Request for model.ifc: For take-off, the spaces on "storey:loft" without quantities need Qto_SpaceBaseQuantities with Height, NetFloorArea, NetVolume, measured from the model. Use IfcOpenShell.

First a look at what the model holds.

```python
import ifcopenshell
import ifcopenshell.util.element
import ifcopenshell.util.unit

model = ifcopenshell.open("model.ifc")
print(model.schema)
for unit_type in ("LENGTHUNIT", "AREAUNIT", "VOLUMEUNIT"):
    print(unit_type, ifcopenshell.util.unit.calculate_unit_scale(model, unit_type))
storey = next(s for s in model.by_type("IfcBuildingStorey") if s.Name == "storey:loft")
spaces = [e for e in ifcopenshell.util.element.get_decomposition(storey) if e.is_a("IfcSpace")]
for e in sorted(spaces, key=lambda e: e.id()):
    print(e.id(), e.is_a(), e.Name, list(ifcopenshell.util.element.get_psets(e, qtos_only=True)), sep=" | ")
```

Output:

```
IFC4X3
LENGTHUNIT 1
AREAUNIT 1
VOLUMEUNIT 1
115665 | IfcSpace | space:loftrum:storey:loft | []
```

```python
import ifcopenshell
import ifcopenshell.api.pset
import ifcopenshell.geom
import ifcopenshell.util.element
import ifcopenshell.util.shape
import ifcopenshell.util.unit

model = ifcopenshell.open("model.ifc")
unit_scale = ifcopenshell.util.unit.calculate_unit_scale(model)
area_scale = ifcopenshell.util.unit.calculate_unit_scale(model, "AREAUNIT")
volume_scale = ifcopenshell.util.unit.calculate_unit_scale(model, "VOLUMEUNIT")
settings = ifcopenshell.geom.settings()

storey = next(s for s in model.by_type("IfcBuildingStorey") if s.Name == "storey:loft")
spaces = [e for e in ifcopenshell.util.element.get_decomposition(storey) if e.is_a("IfcSpace")]

for e in sorted(spaces, key=lambda e: e.id()):
    if ifcopenshell.util.element.get_psets(e, qtos_only=True, should_inherit=False):
        continue
    # Geometry comes back in metres, in the element's own axes.
    shape = ifcopenshell.geom.create_shape(settings, e)
    values = {
        "Height": ifcopenshell.util.shape.get_z(shape.geometry) / unit_scale,
        "NetFloorArea": ifcopenshell.util.shape.get_footprint_area(shape.geometry) / area_scale,
        "NetVolume": ifcopenshell.util.shape.get_volume(shape.geometry) / volume_scale,
    }
    qto = ifcopenshell.api.pset.add_qto(model, product=e, name="Qto_SpaceBaseQuantities")
    ifcopenshell.api.pset.edit_qto(model, qto=qto, properties=values)
    print(e.id(), {k: round(v, 3) for k, v in values.items()})

model.write("model_updated.ifc")
```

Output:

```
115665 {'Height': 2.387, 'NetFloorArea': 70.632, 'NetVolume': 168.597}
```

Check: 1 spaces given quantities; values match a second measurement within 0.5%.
